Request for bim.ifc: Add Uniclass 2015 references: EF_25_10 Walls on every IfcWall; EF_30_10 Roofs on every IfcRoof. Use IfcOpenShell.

First a look at what the model holds.

```python
import ifcopenshell

model = ifcopenshell.open("bim.ifc")
print(model.schema)
print("classifications:", [c.Name for c in model.by_type("IfcClassification")])
for ifc_class in ("IfcDoor", "IfcRoof", "IfcStair", "IfcWall", "IfcWindow"):
    print(ifc_class, len(model.by_type(ifc_class)))
```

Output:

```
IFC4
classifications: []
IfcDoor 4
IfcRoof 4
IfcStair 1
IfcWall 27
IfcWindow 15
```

```python
import ifcopenshell
import ifcopenshell.api.classification

model = ifcopenshell.open("bim.ifc")

system = ifcopenshell.api.classification.add_classification(model, classification="Uniclass 2015")

codes = {
    "IfcWall": ("EF_25_10", "Walls"),
    "IfcRoof": ("EF_30_10", "Roofs"),
}
for ifc_class, (code, name) in codes.items():
    products = model.by_type(ifc_class)
    ifcopenshell.api.classification.add_reference(
        model, products=products, classification=system, identification=code, name=name
    )
    print(code, len(products))

model.write("bim_v2.ifc")
```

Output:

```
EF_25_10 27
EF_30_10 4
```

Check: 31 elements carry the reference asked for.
